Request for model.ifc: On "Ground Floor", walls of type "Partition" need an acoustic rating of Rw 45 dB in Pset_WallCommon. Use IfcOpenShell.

First a look at what the model holds.

```python
import ifcopenshell
import ifcopenshell.util.element

model = ifcopenshell.open("model.ifc")
print(model.schema)
storey = next(s for s in model.by_type("IfcBuildingStorey") if s.Name == "Ground Floor")
walls = [e for e in ifcopenshell.util.element.get_decomposition(storey) if e.is_a("IfcWall")]
seen = {}
for e in walls:
    element_type = ifcopenshell.util.element.get_type(e)
    key = (element_type.Name if element_type != e and element_type else None, ifcopenshell.util.element.get_pset(e, "Pset_WallCommon", "AcousticRating"))
    seen[key] = seen.get(key, 0) + 1
for (name, value), count in sorted(seen.items(), key=str):
    print(count, "x", name, "|", value)
```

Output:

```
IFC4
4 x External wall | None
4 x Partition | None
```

```python
import ifcopenshell
import ifcopenshell.api.pset
import ifcopenshell.util.element

model = ifcopenshell.open("model.ifc")

storey = next(s for s in model.by_type("IfcBuildingStorey") if s.Name == "Ground Floor")
walls = [e for e in ifcopenshell.util.element.get_decomposition(storey) if e.is_a("IfcWall")]

count = 0
for e in walls:
    element_type = ifcopenshell.util.element.get_type(e)
    if element_type in (None, e) or element_type.Name != "Partition":
        continue
    # add_pset returns the element's existing set when there is one.
    pset = ifcopenshell.api.pset.add_pset(model, product=e, name="Pset_WallCommon")
    ifcopenshell.api.pset.edit_pset(model, pset=pset, properties={"AcousticRating": "Rw 45 dB"})
    count += 1

print(count, "walls updated")

model.write("model_rev.ifc")
```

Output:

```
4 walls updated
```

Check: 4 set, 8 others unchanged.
